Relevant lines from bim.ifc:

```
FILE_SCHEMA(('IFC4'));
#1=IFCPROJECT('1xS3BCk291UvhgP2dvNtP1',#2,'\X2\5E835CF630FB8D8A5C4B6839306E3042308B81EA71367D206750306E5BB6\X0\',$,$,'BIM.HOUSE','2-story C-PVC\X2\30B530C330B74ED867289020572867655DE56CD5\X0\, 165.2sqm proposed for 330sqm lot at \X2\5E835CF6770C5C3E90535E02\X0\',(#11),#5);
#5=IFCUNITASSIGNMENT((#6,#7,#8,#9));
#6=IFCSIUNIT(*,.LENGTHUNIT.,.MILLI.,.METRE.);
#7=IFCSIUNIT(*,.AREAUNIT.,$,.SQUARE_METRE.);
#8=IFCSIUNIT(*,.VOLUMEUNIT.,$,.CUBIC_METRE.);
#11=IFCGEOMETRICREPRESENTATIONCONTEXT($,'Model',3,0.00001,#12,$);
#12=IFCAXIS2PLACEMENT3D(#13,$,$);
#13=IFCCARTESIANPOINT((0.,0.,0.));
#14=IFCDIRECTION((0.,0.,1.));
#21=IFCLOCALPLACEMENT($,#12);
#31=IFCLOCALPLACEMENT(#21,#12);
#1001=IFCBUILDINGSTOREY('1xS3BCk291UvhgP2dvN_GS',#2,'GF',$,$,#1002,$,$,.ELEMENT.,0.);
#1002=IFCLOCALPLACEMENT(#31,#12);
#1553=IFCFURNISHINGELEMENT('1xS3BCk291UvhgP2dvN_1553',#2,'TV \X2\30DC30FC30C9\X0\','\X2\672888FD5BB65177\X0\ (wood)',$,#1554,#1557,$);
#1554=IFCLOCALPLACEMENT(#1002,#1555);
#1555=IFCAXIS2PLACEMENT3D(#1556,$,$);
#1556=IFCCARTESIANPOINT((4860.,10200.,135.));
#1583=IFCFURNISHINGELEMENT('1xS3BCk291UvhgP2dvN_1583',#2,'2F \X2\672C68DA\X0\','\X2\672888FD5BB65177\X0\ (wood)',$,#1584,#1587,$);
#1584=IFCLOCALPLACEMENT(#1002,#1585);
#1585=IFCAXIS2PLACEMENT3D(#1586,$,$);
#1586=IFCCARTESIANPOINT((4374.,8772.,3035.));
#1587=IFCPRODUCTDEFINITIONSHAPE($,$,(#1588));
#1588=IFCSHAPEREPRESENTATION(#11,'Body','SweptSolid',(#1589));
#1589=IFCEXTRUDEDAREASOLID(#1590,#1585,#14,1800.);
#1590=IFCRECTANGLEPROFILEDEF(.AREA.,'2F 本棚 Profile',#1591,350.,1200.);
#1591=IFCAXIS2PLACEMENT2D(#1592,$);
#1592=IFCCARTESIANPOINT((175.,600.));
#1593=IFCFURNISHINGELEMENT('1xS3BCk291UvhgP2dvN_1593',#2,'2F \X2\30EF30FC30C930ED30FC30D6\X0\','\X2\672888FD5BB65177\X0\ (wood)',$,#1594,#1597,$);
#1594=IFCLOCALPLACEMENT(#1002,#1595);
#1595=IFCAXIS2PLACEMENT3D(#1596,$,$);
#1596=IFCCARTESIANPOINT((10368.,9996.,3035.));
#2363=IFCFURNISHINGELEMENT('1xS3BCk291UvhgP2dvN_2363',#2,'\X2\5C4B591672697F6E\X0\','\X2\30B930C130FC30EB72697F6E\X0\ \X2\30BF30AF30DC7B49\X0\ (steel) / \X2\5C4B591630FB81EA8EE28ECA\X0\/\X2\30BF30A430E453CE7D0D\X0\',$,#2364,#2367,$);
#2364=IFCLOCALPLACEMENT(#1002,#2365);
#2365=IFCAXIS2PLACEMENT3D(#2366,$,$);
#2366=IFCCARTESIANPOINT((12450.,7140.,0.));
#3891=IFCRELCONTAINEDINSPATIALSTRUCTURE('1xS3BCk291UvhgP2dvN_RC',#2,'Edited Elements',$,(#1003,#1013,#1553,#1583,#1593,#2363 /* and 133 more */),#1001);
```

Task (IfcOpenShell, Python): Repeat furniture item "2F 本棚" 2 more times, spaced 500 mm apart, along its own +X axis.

```python
import ifcopenshell
import ifcopenshell.api.geometry
import ifcopenshell.api.root
import ifcopenshell.util.element
import ifcopenshell.util.placement
import ifcopenshell.util.unit

model = ifcopenshell.open("bim.ifc")
unit_scale = ifcopenshell.util.unit.calculate_unit_scale(model)


def reuse_history(source, copy):
    """copy_class also copies each property set's owner history, people and application; keep the originals."""
    for rel in copy.IsDefinedBy:
        if rel.is_a("IfcRelDefinesByProperties") and (history := rel.RelatingPropertyDefinition.OwnerHistory):
            rel.RelatingPropertyDefinition.OwnerHistory = source.OwnerHistory
            ifcopenshell.util.element.remove_deep2(model, history)


source = model.by_id(1583)
base = ifcopenshell.util.placement.get_local_placement(source.ObjectPlacement)
step = base[:3, 0] * 0.5 / unit_scale

for i in range(1, 3):
    copy = ifcopenshell.api.root.copy_class(model, product=source)
    copy.Representation = ifcopenshell.util.element.copy_deep(
        model, source.Representation, exclude=["IfcGeometricRepresentationContext", "IfcRepresentationMap"]
    )
    reuse_history(source, copy)
    matrix = base.copy()
    matrix[:3, 3] += i * step
    print("added at", matrix[:3, 3].round(3) + 0.0)
    ifcopenshell.api.geometry.edit_object_placement(model, product=copy, matrix=matrix, is_si=False)

model.write("bim_rev.ifc")
```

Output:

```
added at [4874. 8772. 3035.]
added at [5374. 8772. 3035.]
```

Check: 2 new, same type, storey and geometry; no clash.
